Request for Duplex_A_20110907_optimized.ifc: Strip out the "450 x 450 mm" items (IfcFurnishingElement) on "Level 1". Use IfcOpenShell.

First a look at what the model holds.

```python
import ifcopenshell
import ifcopenshell.util.element

model = ifcopenshell.open("Duplex_A_20110907_optimized.ifc")
print(model.schema)
storey = next(s for s in model.by_type("IfcBuildingStorey") if s.Name == "Level 1")
furniture = [e for e in ifcopenshell.util.element.get_decomposition(storey) if e.is_a("IfcFurnishingElement")]
seen = {}
for e in furniture:
    element_type = ifcopenshell.util.element.get_type(e)
    name = element_type.Name if element_type not in (None, e) else None
    seen[name] = seen.get(name, 0) + 1
for name, count in sorted(seen.items(), key=str):
    print(count, "x", name)
```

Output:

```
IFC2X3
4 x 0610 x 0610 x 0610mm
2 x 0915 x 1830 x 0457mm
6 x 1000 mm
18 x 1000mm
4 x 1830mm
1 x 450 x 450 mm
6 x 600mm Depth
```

```python
import ifcopenshell
import ifcopenshell.api.root
import ifcopenshell.util.element

model = ifcopenshell.open("Duplex_A_20110907_optimized.ifc")

storey = next(s for s in model.by_type("IfcBuildingStorey") if s.Name == "Level 1")
furniture = [e for e in ifcopenshell.util.element.get_decomposition(storey) if e.is_a("IfcFurnishingElement")]
targets = [e for e in furniture if (t := ifcopenshell.util.element.get_type(e)) not in (None, e) and t.Name == "450 x 450 mm"]

for e in targets:
    ifcopenshell.api.root.remove_product(model, product=e)
print(len(targets), "removed")

model.write("Duplex_A_20110907_optimized_rev.ifc")
```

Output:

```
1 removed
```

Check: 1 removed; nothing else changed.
